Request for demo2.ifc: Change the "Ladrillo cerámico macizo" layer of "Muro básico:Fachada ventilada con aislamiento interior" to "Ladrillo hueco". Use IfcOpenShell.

First a look at what the model holds.

```python
import ifcopenshell
import ifcopenshell.util.element

model = ifcopenshell.open("demo2.ifc")
print(model.schema)
for layer_set in model.by_type("IfcMaterialLayerSet"):
    if layer_set.LayerSetName == "Muro básico:Fachada ventilada con aislamiento interior":
        for layer in layer_set.MaterialLayers:
            print(layer.id(), layer.Material and layer.Material.Name, layer.LayerThickness, sep=" | ")
        print(len(ifcopenshell.util.element.get_elements_by_material(model, layer_set)), "elements and types use it")
print(sorted(m.Name for m in model.by_type("IfcMaterial") if m.Name)[:60])
```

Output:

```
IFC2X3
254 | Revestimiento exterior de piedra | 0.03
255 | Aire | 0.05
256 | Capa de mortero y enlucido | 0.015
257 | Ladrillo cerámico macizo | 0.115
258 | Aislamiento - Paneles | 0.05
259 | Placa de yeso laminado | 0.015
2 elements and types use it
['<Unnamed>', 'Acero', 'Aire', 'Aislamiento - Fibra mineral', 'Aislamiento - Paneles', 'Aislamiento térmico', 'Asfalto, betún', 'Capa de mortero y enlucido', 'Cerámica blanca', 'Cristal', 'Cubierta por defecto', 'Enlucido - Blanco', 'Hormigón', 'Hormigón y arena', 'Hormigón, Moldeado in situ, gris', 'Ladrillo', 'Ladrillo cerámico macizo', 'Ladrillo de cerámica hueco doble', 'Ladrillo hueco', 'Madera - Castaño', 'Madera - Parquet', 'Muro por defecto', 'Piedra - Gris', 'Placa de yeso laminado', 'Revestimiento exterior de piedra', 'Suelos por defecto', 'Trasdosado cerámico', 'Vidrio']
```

```python
import ifcopenshell
import ifcopenshell.api.material

model = ifcopenshell.open("demo2.ifc")

layer_set = next(s for s in model.by_type("IfcMaterialLayerSet") if s.LayerSetName == "Muro básico:Fachada ventilada con aislamiento interior")
layer = next(l for l in layer_set.MaterialLayers if l.Material and l.Material.Name == "Ladrillo cerámico macizo")
material = next(m for m in model.by_type("IfcMaterial") if m.Name == "Ladrillo hueco")

# Point this one layer at the other material; renaming the old one would change it everywhere.
ifcopenshell.api.material.edit_layer(model, layer=layer, attributes={}, material=material)

print([l.Material.Name if l.Material else None for l in layer_set.MaterialLayers])

model.write("demo2_v2.ifc")
```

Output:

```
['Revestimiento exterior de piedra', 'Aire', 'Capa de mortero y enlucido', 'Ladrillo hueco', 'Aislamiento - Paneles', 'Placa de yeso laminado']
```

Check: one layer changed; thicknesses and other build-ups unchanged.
